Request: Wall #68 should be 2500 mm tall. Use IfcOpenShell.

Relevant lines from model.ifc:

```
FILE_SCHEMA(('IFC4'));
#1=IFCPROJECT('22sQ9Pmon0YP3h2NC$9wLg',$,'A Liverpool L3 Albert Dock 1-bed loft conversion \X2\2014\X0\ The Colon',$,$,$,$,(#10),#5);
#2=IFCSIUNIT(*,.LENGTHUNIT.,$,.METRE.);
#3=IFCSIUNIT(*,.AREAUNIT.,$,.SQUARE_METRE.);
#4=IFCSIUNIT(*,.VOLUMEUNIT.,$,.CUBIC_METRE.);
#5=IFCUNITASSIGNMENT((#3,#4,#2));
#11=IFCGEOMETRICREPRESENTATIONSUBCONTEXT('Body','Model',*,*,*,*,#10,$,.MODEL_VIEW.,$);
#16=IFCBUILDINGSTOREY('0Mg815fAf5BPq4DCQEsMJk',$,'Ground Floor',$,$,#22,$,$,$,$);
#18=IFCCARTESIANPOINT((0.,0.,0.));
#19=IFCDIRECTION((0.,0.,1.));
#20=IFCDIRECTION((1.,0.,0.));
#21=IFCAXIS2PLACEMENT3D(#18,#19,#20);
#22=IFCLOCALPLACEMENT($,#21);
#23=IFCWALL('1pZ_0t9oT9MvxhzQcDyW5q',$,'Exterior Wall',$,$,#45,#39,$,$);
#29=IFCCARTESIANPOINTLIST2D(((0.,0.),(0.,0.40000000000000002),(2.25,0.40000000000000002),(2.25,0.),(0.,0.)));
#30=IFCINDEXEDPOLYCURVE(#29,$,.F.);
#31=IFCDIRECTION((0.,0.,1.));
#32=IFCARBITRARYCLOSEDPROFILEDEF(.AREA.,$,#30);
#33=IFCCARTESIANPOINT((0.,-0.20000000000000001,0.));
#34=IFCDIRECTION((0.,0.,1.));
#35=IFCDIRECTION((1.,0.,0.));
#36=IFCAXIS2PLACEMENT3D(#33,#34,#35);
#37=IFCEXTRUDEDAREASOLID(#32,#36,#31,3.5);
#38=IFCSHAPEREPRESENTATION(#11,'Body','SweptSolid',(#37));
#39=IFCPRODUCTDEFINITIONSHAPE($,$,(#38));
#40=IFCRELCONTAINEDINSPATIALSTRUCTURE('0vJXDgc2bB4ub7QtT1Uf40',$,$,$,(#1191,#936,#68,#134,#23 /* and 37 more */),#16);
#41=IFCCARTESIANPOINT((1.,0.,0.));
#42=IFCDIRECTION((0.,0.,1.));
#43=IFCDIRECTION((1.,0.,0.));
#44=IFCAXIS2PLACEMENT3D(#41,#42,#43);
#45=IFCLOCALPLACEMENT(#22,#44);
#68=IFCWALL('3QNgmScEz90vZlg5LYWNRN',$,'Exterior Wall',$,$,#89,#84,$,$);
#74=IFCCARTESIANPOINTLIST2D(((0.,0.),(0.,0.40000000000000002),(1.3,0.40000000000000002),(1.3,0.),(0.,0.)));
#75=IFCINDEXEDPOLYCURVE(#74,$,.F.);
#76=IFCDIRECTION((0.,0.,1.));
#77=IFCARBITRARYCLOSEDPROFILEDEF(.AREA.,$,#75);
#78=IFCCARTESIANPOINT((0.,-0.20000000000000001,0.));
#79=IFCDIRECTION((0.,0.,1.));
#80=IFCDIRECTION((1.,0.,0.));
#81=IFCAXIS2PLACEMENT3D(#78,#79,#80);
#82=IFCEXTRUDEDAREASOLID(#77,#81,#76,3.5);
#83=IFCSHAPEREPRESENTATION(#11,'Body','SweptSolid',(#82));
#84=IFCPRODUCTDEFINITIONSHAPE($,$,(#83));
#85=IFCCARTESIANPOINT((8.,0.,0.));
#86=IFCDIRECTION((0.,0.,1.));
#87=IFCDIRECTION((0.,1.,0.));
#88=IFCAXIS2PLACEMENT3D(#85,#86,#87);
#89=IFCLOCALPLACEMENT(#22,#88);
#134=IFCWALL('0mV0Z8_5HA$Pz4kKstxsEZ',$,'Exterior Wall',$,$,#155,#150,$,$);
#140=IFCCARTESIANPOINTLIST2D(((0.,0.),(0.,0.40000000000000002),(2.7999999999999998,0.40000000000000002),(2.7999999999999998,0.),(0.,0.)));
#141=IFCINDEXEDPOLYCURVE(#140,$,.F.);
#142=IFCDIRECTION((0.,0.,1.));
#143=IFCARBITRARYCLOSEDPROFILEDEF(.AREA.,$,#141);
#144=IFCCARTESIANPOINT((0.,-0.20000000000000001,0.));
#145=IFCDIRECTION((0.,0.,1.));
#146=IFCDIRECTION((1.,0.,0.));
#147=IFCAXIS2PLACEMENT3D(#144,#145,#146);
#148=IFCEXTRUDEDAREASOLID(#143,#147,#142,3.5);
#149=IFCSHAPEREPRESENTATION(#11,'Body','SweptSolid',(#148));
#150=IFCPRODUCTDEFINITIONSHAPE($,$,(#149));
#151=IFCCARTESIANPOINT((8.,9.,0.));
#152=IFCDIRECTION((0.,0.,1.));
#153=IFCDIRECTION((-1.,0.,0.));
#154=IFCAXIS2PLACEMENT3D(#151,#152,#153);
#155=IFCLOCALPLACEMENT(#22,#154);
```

```python
import ifcopenshell
import ifcopenshell.geom
import ifcopenshell.util.representation
import ifcopenshell.util.shape
import ifcopenshell.util.unit

model = ifcopenshell.open("model.ifc")
unit_scale = ifcopenshell.util.unit.calculate_unit_scale(model)
settings = ifcopenshell.geom.settings()


def volume(element):
    """Net volume in cubic metres, openings subtracted."""
    shape = ifcopenshell.geom.create_shape(settings, element)
    return ifcopenshell.util.shape.get_volume(shape.geometry)


wall = model.by_guid("3QNgmScEz90vZlg5LYWNRN")
before = volume(wall)

body = ifcopenshell.util.representation.get_representation(wall, "Model", "Body")
solid = body.Items[0]
old_height = solid.Depth
solid.Depth = 2.5 / unit_scale
after = volume(wall)

print(f"height {old_height:g} -> {solid.Depth:g}, volume {before:.3f} -> {after:.3f} m3")

model.write("model_updated.ifc")
```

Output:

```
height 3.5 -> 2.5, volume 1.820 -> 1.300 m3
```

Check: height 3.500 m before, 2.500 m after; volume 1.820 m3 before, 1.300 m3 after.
